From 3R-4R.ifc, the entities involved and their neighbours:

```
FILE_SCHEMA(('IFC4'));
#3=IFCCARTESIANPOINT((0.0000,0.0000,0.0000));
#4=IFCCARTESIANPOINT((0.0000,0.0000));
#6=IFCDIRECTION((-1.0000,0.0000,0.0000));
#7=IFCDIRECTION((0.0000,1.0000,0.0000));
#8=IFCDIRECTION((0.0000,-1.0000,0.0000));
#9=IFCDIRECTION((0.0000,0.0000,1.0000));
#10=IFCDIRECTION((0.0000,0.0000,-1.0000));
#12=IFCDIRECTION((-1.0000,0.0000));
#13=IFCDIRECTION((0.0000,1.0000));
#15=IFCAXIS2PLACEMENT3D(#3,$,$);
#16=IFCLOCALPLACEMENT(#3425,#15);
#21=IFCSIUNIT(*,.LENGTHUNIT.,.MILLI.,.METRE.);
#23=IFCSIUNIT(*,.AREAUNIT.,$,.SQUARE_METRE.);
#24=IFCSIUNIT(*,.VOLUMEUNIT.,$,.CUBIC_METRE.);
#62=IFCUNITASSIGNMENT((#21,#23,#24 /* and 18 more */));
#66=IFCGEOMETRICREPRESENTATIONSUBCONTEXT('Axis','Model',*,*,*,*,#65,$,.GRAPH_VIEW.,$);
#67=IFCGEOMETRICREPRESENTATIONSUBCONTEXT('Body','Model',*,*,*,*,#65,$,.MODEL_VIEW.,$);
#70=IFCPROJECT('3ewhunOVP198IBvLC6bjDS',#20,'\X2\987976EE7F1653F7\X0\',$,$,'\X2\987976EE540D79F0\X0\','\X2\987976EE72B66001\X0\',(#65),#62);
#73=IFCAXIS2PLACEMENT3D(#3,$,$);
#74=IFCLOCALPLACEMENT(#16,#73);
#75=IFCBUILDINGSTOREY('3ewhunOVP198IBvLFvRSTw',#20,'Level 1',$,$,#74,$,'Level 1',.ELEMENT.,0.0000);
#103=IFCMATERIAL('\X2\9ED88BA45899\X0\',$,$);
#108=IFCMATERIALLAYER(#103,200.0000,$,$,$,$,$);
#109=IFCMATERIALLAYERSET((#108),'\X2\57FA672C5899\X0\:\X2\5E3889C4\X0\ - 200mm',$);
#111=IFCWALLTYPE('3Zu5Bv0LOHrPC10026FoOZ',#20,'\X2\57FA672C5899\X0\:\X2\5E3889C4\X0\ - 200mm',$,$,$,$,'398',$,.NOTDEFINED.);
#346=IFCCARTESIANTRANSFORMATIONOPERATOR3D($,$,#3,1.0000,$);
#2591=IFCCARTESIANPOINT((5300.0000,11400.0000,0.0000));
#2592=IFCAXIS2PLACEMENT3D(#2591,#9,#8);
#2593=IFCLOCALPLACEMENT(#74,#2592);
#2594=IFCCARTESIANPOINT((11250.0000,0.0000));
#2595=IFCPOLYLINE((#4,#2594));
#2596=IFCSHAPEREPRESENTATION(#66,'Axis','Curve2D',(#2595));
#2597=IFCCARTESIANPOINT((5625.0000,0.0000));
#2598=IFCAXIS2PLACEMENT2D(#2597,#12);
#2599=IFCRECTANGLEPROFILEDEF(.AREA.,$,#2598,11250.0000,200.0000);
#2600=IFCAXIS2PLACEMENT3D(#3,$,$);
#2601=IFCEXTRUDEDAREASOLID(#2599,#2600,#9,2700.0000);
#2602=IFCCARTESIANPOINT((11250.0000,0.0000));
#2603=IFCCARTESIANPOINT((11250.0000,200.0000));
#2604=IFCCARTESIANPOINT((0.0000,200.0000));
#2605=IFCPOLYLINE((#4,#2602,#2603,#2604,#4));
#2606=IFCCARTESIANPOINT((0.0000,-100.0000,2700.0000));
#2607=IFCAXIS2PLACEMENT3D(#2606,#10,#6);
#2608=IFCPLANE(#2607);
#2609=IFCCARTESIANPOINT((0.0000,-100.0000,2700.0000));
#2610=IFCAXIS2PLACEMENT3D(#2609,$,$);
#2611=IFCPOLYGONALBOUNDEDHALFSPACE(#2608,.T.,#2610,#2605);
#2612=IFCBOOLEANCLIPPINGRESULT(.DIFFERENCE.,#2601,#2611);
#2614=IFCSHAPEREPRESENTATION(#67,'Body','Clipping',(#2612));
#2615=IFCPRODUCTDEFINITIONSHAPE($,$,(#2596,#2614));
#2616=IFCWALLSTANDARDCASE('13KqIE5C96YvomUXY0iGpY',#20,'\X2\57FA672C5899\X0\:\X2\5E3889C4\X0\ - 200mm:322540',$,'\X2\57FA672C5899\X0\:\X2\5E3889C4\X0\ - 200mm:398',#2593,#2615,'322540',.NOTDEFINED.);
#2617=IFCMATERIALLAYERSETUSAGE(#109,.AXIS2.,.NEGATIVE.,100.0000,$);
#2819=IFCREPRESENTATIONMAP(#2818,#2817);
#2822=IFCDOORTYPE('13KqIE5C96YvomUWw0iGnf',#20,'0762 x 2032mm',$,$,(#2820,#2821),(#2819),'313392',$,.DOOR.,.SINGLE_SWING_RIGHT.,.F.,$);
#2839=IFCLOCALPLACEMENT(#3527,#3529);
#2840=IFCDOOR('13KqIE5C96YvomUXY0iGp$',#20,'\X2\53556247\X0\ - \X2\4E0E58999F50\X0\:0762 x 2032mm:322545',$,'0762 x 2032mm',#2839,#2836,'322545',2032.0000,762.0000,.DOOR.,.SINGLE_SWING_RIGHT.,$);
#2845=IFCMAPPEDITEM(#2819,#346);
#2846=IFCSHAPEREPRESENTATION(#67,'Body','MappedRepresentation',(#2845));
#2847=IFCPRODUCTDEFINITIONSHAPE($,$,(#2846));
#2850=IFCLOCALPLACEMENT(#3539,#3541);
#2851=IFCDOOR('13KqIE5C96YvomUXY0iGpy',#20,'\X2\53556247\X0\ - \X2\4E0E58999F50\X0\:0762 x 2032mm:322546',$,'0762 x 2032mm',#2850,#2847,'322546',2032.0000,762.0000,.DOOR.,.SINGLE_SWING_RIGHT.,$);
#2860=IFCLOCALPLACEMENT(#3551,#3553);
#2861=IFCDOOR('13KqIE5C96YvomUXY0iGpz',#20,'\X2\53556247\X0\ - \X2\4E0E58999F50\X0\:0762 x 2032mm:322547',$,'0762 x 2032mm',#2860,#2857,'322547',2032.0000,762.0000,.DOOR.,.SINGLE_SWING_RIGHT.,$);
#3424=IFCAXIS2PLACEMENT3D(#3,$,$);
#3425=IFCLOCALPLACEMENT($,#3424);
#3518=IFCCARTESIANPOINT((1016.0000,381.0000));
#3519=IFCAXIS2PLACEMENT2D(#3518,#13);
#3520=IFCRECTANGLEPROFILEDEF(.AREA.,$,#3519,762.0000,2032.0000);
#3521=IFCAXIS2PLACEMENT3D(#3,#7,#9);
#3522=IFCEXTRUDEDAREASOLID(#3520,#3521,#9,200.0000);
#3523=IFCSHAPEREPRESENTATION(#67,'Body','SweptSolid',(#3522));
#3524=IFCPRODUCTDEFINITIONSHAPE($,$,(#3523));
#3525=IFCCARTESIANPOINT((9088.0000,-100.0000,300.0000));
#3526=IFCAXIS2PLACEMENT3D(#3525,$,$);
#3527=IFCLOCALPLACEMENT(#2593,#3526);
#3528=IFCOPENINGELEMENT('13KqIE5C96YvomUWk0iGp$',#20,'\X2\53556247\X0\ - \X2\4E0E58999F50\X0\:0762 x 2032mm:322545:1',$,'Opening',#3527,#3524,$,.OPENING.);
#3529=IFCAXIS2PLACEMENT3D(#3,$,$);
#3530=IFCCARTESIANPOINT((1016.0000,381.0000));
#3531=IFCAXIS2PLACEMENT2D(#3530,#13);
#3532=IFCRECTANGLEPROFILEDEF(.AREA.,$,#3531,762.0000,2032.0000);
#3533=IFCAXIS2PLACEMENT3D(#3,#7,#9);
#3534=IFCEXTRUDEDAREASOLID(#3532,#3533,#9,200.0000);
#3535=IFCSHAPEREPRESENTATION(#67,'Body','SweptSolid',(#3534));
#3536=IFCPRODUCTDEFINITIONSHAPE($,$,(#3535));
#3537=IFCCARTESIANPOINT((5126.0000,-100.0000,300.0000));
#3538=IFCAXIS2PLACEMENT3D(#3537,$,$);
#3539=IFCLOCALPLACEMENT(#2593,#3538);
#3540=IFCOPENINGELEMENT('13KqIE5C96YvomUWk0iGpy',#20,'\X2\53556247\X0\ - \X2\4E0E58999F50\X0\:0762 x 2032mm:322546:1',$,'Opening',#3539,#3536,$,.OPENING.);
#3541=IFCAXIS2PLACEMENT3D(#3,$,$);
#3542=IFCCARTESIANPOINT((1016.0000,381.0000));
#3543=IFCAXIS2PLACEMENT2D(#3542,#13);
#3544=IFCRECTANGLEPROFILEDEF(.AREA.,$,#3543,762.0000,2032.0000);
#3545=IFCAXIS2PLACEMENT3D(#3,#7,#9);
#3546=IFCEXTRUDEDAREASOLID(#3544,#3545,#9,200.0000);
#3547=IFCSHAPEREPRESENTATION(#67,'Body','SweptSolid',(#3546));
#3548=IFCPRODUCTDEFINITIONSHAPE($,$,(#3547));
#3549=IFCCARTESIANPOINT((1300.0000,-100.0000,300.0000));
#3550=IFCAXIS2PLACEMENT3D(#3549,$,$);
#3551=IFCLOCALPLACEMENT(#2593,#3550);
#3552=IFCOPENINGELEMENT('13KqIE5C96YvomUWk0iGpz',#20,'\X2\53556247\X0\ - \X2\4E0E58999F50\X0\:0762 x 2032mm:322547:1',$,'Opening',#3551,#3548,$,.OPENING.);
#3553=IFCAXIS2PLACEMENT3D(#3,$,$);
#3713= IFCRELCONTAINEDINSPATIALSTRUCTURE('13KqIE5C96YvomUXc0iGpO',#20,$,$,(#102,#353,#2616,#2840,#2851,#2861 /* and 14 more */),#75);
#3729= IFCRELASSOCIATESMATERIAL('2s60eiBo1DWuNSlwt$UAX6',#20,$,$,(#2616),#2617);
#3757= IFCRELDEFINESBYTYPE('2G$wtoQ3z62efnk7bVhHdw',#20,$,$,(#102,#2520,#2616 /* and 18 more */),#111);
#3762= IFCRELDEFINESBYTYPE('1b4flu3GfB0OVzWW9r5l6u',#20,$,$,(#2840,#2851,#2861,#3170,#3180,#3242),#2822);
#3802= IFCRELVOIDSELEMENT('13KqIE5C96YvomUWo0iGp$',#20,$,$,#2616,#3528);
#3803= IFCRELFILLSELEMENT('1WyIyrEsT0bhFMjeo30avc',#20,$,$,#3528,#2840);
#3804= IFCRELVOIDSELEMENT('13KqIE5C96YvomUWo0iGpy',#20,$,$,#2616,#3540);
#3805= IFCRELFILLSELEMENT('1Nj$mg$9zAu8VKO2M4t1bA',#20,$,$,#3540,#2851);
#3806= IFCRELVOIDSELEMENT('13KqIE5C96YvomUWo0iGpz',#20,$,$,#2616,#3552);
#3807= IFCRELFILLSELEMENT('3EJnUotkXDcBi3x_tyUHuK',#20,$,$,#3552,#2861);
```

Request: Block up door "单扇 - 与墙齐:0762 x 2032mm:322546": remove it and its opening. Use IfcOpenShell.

```python
import ifcopenshell
import ifcopenshell.api.feature
import ifcopenshell.api.root
import ifcopenshell.geom
import ifcopenshell.util.shape

model = ifcopenshell.open("3R-4R.ifc")
settings = ifcopenshell.geom.settings()


def volume(element):
    """Net volume in cubic metres, openings subtracted."""
    shape = ifcopenshell.geom.create_shape(settings, element)
    return ifcopenshell.util.shape.get_volume(shape.geometry)


door = model.by_guid("13KqIE5C96YvomUXY0iGpy")
opening = door.FillsVoids[0].RelatingOpeningElement
wall = opening.VoidsElements[0].RelatingBuildingElement
before = volume(wall)

ifcopenshell.api.root.remove_product(model, product=door)
ifcopenshell.api.feature.remove_feature(model, feature=opening)

after = volume(wall)

print(f"wall volume {before:.3f} -> {after:.3f} m3")

model.write("3R-4R-out.ifc")
```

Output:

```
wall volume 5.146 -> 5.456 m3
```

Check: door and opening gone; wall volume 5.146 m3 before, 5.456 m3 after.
